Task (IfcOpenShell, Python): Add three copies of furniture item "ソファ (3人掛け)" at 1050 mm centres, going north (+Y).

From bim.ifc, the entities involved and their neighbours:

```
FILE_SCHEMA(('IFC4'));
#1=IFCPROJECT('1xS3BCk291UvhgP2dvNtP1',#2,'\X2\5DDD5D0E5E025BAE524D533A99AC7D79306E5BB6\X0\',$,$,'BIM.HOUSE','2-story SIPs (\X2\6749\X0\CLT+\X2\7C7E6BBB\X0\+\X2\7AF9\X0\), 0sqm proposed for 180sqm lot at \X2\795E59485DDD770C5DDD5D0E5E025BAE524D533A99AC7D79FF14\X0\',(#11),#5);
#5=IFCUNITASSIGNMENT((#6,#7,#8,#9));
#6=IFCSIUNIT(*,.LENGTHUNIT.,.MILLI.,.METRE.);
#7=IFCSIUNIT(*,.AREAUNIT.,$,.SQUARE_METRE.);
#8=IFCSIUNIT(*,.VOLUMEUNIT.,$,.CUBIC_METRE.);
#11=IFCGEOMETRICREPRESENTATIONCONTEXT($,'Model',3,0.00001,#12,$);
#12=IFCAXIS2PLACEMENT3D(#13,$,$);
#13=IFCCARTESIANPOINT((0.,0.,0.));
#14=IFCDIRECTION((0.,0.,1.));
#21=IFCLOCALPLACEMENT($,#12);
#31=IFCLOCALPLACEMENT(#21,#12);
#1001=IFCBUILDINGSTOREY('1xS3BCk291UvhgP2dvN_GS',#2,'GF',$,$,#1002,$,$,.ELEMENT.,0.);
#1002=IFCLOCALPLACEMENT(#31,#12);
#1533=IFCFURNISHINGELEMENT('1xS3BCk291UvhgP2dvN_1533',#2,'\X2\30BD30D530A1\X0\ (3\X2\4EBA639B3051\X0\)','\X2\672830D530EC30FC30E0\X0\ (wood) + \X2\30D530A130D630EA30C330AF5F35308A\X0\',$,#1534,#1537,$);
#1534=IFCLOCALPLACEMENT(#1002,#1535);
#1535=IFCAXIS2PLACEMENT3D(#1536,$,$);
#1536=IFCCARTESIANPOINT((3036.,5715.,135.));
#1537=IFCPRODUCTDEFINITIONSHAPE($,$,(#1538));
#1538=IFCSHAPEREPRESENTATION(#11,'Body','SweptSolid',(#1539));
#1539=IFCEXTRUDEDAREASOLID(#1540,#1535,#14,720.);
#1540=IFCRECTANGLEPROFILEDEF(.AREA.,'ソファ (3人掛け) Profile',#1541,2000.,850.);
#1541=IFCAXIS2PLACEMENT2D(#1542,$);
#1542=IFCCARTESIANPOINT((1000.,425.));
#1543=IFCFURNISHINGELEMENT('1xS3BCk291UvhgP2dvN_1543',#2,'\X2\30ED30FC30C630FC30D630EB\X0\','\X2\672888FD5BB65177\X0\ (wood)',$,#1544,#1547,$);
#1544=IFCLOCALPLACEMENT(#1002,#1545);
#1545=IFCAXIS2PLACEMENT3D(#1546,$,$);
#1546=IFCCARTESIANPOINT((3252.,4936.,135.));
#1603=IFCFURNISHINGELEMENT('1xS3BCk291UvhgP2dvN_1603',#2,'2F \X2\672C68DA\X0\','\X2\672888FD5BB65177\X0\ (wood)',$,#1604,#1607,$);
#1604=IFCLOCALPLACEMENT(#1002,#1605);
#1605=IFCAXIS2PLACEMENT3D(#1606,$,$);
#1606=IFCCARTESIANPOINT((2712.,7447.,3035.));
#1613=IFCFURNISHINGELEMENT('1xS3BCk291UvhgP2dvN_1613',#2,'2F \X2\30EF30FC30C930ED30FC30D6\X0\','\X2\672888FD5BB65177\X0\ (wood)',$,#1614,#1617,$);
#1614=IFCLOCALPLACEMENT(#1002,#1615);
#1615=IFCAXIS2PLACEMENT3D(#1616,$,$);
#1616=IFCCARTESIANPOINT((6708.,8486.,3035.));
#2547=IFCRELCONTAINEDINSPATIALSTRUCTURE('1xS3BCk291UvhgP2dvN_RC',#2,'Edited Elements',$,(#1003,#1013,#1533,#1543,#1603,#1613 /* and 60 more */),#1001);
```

```python
import numpy as np
import ifcopenshell
import ifcopenshell.api.geometry
import ifcopenshell.api.root
import ifcopenshell.util.element
import ifcopenshell.util.placement
import ifcopenshell.util.unit

model = ifcopenshell.open("bim.ifc")
unit_scale = ifcopenshell.util.unit.calculate_unit_scale(model)


def reuse_history(source, copy):
    """copy_class also copies each property set's owner history, people and application; keep the originals."""
    for rel in copy.IsDefinedBy:
        if rel.is_a("IfcRelDefinesByProperties") and (history := rel.RelatingPropertyDefinition.OwnerHistory):
            rel.RelatingPropertyDefinition.OwnerHistory = source.OwnerHistory
            ifcopenshell.util.element.remove_deep2(model, history)


source = model.by_guid("1xS3BCk291UvhgP2dvN_1533")
base = ifcopenshell.util.placement.get_local_placement(source.ObjectPlacement)
step = np.array([0.0, 1.0, 0.0]) * 1.05 / unit_scale

for i in range(1, 4):
    copy = ifcopenshell.api.root.copy_class(model, product=source)
    copy.Representation = ifcopenshell.util.element.copy_deep(
        model, source.Representation, exclude=["IfcGeometricRepresentationContext", "IfcRepresentationMap"]
    )
    reuse_history(source, copy)
    matrix = base.copy()
    matrix[:3, 3] += i * step
    print("added at", matrix[:3, 3].round(3) + 0.0)
    ifcopenshell.api.geometry.edit_object_placement(model, product=copy, matrix=matrix, is_si=False)

model.write("bim_v2.ifc")
```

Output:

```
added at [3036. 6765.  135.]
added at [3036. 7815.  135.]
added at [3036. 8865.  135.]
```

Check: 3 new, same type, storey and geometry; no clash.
